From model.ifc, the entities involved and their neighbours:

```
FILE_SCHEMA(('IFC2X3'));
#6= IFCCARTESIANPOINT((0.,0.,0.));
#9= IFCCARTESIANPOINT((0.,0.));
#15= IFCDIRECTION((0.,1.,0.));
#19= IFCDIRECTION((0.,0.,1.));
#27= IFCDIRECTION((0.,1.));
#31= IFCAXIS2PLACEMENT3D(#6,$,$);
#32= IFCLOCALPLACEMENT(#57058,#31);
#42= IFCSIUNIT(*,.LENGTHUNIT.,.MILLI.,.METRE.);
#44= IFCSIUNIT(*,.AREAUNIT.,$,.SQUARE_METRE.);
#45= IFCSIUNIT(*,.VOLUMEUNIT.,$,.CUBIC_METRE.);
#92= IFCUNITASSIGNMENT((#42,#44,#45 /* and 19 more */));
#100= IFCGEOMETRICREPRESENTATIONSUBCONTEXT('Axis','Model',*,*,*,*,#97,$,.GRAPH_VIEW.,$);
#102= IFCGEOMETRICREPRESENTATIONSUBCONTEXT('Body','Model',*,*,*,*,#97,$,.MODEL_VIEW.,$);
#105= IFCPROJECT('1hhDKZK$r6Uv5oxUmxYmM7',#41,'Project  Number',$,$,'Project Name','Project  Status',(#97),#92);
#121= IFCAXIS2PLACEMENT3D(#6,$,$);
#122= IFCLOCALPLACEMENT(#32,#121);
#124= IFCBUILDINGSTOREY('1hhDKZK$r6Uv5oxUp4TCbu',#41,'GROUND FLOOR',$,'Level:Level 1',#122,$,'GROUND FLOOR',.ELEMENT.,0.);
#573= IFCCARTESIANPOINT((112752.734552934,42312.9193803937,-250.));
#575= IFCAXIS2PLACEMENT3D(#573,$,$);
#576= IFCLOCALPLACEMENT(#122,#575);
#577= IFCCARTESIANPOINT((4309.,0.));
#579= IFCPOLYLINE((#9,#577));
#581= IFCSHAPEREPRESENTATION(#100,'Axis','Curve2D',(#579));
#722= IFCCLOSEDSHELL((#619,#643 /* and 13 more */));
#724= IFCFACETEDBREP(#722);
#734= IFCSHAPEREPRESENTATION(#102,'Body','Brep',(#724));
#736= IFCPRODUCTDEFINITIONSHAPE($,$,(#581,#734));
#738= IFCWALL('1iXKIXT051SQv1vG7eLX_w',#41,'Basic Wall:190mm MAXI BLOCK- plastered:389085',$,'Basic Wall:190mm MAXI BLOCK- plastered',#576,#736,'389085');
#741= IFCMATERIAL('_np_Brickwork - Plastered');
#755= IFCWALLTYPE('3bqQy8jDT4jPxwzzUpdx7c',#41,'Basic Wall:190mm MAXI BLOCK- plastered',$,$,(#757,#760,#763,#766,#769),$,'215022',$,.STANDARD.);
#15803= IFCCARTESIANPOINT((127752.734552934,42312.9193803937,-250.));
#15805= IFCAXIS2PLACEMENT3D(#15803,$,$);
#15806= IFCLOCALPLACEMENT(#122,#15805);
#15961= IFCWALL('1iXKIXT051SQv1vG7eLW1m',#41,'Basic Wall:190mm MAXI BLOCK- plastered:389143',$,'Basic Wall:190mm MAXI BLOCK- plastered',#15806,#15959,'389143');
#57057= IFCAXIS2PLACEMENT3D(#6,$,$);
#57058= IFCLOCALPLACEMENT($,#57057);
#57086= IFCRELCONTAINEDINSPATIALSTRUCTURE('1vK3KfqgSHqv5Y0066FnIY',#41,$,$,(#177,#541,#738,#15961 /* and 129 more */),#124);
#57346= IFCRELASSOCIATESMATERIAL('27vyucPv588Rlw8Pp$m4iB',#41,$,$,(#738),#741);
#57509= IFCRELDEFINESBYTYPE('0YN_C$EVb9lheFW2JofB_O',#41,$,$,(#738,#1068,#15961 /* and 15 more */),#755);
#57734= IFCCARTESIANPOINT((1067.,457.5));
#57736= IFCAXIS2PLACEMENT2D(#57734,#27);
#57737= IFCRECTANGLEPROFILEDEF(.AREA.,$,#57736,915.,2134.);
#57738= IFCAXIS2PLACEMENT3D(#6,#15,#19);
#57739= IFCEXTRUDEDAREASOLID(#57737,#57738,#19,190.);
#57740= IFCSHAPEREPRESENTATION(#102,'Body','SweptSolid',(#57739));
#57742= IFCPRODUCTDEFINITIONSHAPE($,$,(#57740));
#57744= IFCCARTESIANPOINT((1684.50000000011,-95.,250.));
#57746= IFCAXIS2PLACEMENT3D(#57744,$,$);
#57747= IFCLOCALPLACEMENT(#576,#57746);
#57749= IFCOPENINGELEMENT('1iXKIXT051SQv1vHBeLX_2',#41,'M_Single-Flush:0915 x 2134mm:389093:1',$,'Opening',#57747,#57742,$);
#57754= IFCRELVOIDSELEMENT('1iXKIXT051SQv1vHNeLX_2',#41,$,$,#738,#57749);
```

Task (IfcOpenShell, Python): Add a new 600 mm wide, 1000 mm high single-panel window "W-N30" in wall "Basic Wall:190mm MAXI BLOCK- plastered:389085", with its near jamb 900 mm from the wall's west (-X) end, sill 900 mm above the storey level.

```python
import numpy as np
import ifcopenshell
import ifcopenshell.api.feature
import ifcopenshell.api.geometry
import ifcopenshell.api.root
import ifcopenshell.api.spatial
import ifcopenshell.api.type
import ifcopenshell.geom
import ifcopenshell.util.element
import ifcopenshell.util.placement
import ifcopenshell.util.representation
import ifcopenshell.util.shape
import ifcopenshell.util.unit

model = ifcopenshell.open("model.ifc")
unit_scale = ifcopenshell.util.unit.calculate_unit_scale(model)
settings = ifcopenshell.geom.settings()


def volume(element):
    """Net volume in cubic metres, openings subtracted."""
    shape = ifcopenshell.geom.create_shape(settings, element)
    return ifcopenshell.util.shape.get_volume(shape.geometry)


wall = model.by_guid("1iXKIXT051SQv1vG7eLX_w")
storey = ifcopenshell.util.element.get_container(wall, ifc_class="IfcBuildingStorey")
context = ifcopenshell.util.representation.get_context(model, "Model", "Body", "MODEL_VIEW")
before = volume(wall)

width, height, from_end, sill = 0.6, 1, 0.9, 0.9  # metres

# The wall runs along its own X axis, and the end named is its -X end.
wall_shape = ifcopenshell.geom.create_shape(settings, wall)
x, y, z = ifcopenshell.util.shape.get_vertices(wall_shape.geometry).T
start = x.min() + from_end
face, thickness = float(y.min()), float(y.max() - y.min())
wall_matrix = ifcopenshell.util.placement.get_local_placement(wall.ObjectPlacement)
level = ifcopenshell.util.placement.get_local_placement(storey.ObjectPlacement)[2, 3]


def in_wall(x, y):
    """Placement at x, y metres in the wall's axes, at sill height."""
    matrix = wall_matrix.copy()
    matrix[:, 3] = wall_matrix @ np.array([x / unit_scale, y / unit_scale, 0.0, 1.0])
    matrix[2, 3] = level + sill / unit_scale
    return matrix


# Opening: a box that overshoots both wall faces by 50 mm.
opening = ifcopenshell.api.root.create_entity(model, ifc_class="IfcOpeningElement")
box = ifcopenshell.api.geometry.add_wall_representation(
    model, context=context, length=width, height=height, thickness=thickness + 0.1
)
ifcopenshell.api.geometry.assign_representation(model, product=opening, representation=box)
ifcopenshell.api.geometry.edit_object_placement(model, product=opening, matrix=in_wall(start, face - 0.05), is_si=False)
ifcopenshell.api.feature.add_feature(model, feature=opening, element=wall)

window = ifcopenshell.api.root.create_entity(model, ifc_class="IfcWindow", name="W-N30")
window.OverallWidth, window.OverallHeight = width / unit_scale, height / unit_scale
body = ifcopenshell.api.geometry.add_window_representation(
    model,
    context=context,
    overall_width=window.OverallWidth,
    overall_height=window.OverallHeight,
    partition_type="SINGLE_PANEL",
)
ifcopenshell.api.geometry.assign_representation(model, product=window, representation=body)
ifcopenshell.api.spatial.assign_container(model, products=[window], relating_structure=storey)
fills = ifcopenshell.api.feature.add_filling(model, opening=opening, element=window)
fills.OwnerHistory = window.OwnerHistory  # required in IFC2X3

# IFC2X3 keeps the operation on the window style.
style = ifcopenshell.api.root.create_entity(model, ifc_class="IfcWindowStyle", name="W-N30")
style.OperationType, style.ConstructionType = "SINGLE_PANEL", "NOTDEFINED"
style.ParameterTakesPrecedence = style.Sizeable = False
ifcopenshell.api.type.assign_type(model, related_objects=[window], relating_type=style)

# Centre the window in the wall's thickness.
ifcopenshell.api.geometry.edit_object_placement(model, product=window, matrix=in_wall(start, face), is_si=False)
window_shape = ifcopenshell.geom.create_shape(settings, window)
depth = ifcopenshell.util.shape.get_vertices(window_shape.geometry)[:, 1]
offset = face + thickness / 2 - (depth.min() + depth.max()) / 2
ifcopenshell.api.geometry.edit_object_placement(model, product=window, matrix=in_wall(start, offset), is_si=False)

after = volume(wall)

print(f"wall volume {before:.3f} -> {after:.3f} m3")

model.write("model-out.ifc")
```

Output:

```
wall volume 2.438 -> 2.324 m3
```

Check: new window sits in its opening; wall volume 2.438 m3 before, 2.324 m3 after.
